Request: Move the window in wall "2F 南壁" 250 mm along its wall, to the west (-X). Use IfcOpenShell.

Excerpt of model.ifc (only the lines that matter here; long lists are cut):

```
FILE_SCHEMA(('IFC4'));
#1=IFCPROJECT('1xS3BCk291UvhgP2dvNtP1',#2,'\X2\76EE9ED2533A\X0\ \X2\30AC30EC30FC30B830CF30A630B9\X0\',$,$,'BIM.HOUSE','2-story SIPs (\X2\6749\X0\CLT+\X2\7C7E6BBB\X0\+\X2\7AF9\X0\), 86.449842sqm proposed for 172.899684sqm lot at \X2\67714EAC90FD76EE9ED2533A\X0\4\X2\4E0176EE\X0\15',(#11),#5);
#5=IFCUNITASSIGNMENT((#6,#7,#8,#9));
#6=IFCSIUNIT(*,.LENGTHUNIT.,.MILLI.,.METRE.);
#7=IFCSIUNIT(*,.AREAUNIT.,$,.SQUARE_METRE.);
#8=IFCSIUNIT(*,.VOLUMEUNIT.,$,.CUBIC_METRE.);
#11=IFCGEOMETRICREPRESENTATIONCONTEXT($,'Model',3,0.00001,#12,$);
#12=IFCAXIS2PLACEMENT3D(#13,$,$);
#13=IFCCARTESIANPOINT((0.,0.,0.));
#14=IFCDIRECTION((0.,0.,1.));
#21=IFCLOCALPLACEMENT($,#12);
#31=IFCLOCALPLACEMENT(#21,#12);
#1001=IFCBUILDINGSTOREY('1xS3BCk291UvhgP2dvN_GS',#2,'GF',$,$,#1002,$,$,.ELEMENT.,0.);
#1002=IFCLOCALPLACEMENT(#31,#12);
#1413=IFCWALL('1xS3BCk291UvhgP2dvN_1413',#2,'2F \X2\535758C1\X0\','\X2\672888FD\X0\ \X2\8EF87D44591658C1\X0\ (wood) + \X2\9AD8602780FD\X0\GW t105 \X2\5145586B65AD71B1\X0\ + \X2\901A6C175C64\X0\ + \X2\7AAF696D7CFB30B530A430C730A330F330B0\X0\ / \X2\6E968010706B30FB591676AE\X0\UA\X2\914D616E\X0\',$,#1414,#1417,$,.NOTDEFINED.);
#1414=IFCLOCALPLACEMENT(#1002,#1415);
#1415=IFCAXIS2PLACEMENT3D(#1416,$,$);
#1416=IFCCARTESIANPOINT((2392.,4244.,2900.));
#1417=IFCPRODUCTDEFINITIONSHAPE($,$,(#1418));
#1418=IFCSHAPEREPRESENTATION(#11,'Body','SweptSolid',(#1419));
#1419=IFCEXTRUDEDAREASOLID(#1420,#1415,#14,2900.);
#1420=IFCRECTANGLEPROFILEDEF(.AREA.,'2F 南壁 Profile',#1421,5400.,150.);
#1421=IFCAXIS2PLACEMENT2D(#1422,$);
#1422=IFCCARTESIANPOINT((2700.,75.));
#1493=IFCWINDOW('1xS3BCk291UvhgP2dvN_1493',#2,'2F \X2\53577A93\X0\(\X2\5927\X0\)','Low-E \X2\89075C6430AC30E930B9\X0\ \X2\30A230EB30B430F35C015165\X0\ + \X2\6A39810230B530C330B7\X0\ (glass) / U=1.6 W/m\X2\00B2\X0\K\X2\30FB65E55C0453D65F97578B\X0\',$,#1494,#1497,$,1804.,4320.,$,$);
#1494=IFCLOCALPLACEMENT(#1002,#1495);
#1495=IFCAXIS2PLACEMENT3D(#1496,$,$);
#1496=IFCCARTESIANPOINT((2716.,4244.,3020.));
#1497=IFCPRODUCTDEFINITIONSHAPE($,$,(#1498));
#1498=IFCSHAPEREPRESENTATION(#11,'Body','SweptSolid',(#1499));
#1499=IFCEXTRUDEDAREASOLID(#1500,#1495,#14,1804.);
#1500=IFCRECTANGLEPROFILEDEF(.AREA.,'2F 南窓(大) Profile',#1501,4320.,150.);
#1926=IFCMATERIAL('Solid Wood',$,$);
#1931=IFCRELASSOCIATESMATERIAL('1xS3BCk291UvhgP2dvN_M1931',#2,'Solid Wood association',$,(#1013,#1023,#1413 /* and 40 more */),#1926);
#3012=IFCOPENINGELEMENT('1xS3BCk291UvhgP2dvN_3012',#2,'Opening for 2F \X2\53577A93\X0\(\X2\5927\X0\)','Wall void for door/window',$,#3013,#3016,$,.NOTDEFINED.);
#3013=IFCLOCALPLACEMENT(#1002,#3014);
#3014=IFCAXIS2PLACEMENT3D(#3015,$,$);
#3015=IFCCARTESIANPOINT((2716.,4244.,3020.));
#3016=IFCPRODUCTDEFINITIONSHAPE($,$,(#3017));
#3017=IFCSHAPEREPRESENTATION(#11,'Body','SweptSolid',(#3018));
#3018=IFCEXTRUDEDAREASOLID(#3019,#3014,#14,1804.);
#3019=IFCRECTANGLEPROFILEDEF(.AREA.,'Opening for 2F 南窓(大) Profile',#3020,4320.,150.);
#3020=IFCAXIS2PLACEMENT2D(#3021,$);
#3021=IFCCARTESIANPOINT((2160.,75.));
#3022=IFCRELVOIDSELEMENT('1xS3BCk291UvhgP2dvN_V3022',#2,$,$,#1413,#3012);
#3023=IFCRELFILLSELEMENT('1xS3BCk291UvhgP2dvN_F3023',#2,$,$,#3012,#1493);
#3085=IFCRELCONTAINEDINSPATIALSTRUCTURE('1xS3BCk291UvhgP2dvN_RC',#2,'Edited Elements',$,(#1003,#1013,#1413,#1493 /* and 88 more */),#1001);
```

```python
import ifcopenshell
import ifcopenshell.api.geometry
import ifcopenshell.util.placement
import ifcopenshell.util.unit

model = ifcopenshell.open("model.ifc")
unit_scale = ifcopenshell.util.unit.calculate_unit_scale(model)

window = model.by_guid("1xS3BCk291UvhgP2dvN_1493")
opening = window.FillsVoids[0].RelatingOpeningElement
wall = opening.VoidsElements[0].RelatingBuildingElement

wall_matrix = ifcopenshell.util.placement.get_local_placement(wall.ObjectPlacement)
shift = wall_matrix[:3, 0] * -0.25 / unit_scale
before = ifcopenshell.util.placement.get_local_placement(window.ObjectPlacement)[:3, 3].copy()

# The window is not placed relative to its opening, so move both.
for product in (opening, window):
    matrix = ifcopenshell.util.placement.get_local_placement(product.ObjectPlacement)
    matrix[:3, 3] += shift
    ifcopenshell.api.geometry.edit_object_placement(model, product=product, matrix=matrix, is_si=False)

after = ifcopenshell.util.placement.get_local_placement(window.ObjectPlacement)[:3, 3]
print("window moved by", (after - before).round(3) + 0.0)

model.write("model_v2.ifc")
```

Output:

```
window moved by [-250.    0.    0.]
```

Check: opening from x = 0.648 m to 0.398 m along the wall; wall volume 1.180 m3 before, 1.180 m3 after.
